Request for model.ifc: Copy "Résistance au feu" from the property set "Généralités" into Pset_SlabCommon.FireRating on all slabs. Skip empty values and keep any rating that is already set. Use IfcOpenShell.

First a look at what the model holds.

```python
import ifcopenshell
import ifcopenshell.util.element

model = ifcopenshell.open("model.ifc")
print(model.schema)
slabs = model.by_type("IfcSlab")
print(len(slabs), "slabs")
for e in slabs[:8]:
    source = ifcopenshell.util.element.get_pset(e, "Généralités", "Résistance au feu")
    target = ifcopenshell.util.element.get_pset(e, "Pset_SlabCommon", "FireRating")
    print(e.id(), repr(source), repr(target), sep=" | ")
```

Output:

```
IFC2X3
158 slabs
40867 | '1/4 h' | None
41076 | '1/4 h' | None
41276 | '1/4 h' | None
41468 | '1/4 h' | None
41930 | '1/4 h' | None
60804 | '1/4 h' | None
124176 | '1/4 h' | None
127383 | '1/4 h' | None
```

```python
import ifcopenshell
import ifcopenshell.api.pset
import ifcopenshell.util.element

model = ifcopenshell.open("model.ifc")

count = 0
for e in model.by_type("IfcSlab"):
    value = ifcopenshell.util.element.get_pset(e, "Généralités", "Résistance au feu")
    current = ifcopenshell.util.element.get_pset(e, "Pset_SlabCommon", "FireRating")
    if not value or not value.strip() or current:
        continue
    # add_pset returns the element's existing set when there is one.
    pset = ifcopenshell.api.pset.add_pset(model, product=e, name="Pset_SlabCommon")
    ifcopenshell.api.pset.edit_pset(model, pset=pset, properties={"FireRating": value})
    count += 1

print(count, "slabs updated")

model.write("model_edited.ifc")
```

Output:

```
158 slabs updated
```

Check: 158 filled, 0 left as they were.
